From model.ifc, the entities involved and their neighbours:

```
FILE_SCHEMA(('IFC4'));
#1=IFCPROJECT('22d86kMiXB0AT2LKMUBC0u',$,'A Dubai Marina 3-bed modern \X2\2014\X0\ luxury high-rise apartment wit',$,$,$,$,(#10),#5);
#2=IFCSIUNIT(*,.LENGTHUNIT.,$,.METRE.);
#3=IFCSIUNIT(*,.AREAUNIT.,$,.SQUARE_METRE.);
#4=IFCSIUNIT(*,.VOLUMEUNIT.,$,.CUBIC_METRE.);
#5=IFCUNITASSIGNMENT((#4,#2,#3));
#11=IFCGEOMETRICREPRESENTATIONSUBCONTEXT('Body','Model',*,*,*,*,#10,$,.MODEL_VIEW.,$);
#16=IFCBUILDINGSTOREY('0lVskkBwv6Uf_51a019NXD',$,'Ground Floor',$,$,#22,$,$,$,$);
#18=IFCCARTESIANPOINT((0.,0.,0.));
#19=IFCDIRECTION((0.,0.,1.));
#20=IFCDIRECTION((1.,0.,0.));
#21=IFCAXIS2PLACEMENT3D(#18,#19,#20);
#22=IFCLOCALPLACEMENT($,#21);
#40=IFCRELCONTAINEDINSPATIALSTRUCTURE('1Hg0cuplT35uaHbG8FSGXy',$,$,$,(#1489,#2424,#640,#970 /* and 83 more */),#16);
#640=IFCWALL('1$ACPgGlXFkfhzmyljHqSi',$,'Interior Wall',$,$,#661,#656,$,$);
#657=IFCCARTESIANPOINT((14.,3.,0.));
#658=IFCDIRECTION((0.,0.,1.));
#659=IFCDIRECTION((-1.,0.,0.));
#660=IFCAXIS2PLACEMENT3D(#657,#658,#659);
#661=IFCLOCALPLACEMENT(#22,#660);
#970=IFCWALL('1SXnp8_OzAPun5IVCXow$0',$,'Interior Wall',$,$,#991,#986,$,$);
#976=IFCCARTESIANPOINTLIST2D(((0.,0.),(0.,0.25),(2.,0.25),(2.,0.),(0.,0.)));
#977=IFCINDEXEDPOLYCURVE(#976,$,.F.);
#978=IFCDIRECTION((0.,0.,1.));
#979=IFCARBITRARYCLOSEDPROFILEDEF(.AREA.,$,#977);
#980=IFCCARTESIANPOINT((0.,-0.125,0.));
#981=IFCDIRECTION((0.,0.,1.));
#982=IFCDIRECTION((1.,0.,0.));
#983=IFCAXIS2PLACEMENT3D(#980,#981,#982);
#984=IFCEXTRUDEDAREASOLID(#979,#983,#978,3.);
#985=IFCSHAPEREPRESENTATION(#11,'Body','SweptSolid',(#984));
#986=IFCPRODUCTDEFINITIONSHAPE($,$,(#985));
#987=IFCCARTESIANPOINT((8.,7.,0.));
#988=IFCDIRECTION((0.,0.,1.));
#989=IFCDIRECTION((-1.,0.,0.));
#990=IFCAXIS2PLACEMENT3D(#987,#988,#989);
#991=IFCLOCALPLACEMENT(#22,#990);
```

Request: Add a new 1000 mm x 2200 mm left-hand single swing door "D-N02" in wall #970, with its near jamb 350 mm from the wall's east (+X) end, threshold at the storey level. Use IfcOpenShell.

```python
import numpy as np
import ifcopenshell
import ifcopenshell.api.feature
import ifcopenshell.api.geometry
import ifcopenshell.api.root
import ifcopenshell.api.spatial
import ifcopenshell.geom
import ifcopenshell.util.element
import ifcopenshell.util.placement
import ifcopenshell.util.representation
import ifcopenshell.util.shape
import ifcopenshell.util.unit

model = ifcopenshell.open("model.ifc")
unit_scale = ifcopenshell.util.unit.calculate_unit_scale(model)
settings = ifcopenshell.geom.settings()


def volume(element):
    """Net volume in cubic metres, openings subtracted."""
    shape = ifcopenshell.geom.create_shape(settings, element)
    return ifcopenshell.util.shape.get_volume(shape.geometry)


wall = model.by_guid("1SXnp8_OzAPun5IVCXow$0")
storey = ifcopenshell.util.element.get_container(wall, ifc_class="IfcBuildingStorey")
context = ifcopenshell.util.representation.get_context(model, "Model", "Body", "MODEL_VIEW")
before = volume(wall)

width, height, from_end, sill = 1, 2.2, 0.35, 0.0  # metres

# The wall runs along its own X axis, and the end named is its -X end.
wall_shape = ifcopenshell.geom.create_shape(settings, wall)
x, y, z = ifcopenshell.util.shape.get_vertices(wall_shape.geometry).T
start = x.min() + from_end
face, thickness = float(y.min()), float(y.max() - y.min())
wall_matrix = ifcopenshell.util.placement.get_local_placement(wall.ObjectPlacement)
level = ifcopenshell.util.placement.get_local_placement(storey.ObjectPlacement)[2, 3]


def in_wall(x, y):
    """Placement at x, y metres in the wall's axes, at sill height."""
    matrix = wall_matrix.copy()
    matrix[:, 3] = wall_matrix @ np.array([x / unit_scale, y / unit_scale, 0.0, 1.0])
    matrix[2, 3] = level + sill / unit_scale
    return matrix


# Opening: a box that overshoots both wall faces by 50 mm.
opening = ifcopenshell.api.root.create_entity(model, ifc_class="IfcOpeningElement", predefined_type="OPENING")
box = ifcopenshell.api.geometry.add_wall_representation(
    model, context=context, length=width, height=height, thickness=thickness + 0.1
)
ifcopenshell.api.geometry.assign_representation(model, product=opening, representation=box)
ifcopenshell.api.geometry.edit_object_placement(model, product=opening, matrix=in_wall(start, face - 0.05), is_si=False)
ifcopenshell.api.feature.add_feature(model, feature=opening, element=wall)

door = ifcopenshell.api.root.create_entity(model, ifc_class="IfcDoor", name="D-N02", predefined_type="DOOR")
door.OverallWidth, door.OverallHeight = width / unit_scale, height / unit_scale
door.OperationType = "SINGLE_SWING_LEFT"
body = ifcopenshell.api.geometry.add_door_representation(
    model,
    context=context,
    overall_width=door.OverallWidth,
    overall_height=door.OverallHeight,
    operation_type="SINGLE_SWING_LEFT",
    lining_properties={"LiningDepth": thickness / unit_scale, "ThresholdDepth": thickness / unit_scale},
)
ifcopenshell.api.geometry.assign_representation(model, product=door, representation=body)
ifcopenshell.api.spatial.assign_container(model, products=[door], relating_structure=storey)
ifcopenshell.api.feature.add_filling(model, opening=opening, element=door)

# The lining spans the wall, so the door starts at the wall face.
ifcopenshell.api.geometry.edit_object_placement(model, product=door, matrix=in_wall(start, face), is_si=False)

after = volume(wall)

print(f"wall volume {before:.3f} -> {after:.3f} m3")

model.write("model_edited.ifc")
```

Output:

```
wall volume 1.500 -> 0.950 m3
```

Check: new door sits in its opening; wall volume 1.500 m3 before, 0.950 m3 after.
